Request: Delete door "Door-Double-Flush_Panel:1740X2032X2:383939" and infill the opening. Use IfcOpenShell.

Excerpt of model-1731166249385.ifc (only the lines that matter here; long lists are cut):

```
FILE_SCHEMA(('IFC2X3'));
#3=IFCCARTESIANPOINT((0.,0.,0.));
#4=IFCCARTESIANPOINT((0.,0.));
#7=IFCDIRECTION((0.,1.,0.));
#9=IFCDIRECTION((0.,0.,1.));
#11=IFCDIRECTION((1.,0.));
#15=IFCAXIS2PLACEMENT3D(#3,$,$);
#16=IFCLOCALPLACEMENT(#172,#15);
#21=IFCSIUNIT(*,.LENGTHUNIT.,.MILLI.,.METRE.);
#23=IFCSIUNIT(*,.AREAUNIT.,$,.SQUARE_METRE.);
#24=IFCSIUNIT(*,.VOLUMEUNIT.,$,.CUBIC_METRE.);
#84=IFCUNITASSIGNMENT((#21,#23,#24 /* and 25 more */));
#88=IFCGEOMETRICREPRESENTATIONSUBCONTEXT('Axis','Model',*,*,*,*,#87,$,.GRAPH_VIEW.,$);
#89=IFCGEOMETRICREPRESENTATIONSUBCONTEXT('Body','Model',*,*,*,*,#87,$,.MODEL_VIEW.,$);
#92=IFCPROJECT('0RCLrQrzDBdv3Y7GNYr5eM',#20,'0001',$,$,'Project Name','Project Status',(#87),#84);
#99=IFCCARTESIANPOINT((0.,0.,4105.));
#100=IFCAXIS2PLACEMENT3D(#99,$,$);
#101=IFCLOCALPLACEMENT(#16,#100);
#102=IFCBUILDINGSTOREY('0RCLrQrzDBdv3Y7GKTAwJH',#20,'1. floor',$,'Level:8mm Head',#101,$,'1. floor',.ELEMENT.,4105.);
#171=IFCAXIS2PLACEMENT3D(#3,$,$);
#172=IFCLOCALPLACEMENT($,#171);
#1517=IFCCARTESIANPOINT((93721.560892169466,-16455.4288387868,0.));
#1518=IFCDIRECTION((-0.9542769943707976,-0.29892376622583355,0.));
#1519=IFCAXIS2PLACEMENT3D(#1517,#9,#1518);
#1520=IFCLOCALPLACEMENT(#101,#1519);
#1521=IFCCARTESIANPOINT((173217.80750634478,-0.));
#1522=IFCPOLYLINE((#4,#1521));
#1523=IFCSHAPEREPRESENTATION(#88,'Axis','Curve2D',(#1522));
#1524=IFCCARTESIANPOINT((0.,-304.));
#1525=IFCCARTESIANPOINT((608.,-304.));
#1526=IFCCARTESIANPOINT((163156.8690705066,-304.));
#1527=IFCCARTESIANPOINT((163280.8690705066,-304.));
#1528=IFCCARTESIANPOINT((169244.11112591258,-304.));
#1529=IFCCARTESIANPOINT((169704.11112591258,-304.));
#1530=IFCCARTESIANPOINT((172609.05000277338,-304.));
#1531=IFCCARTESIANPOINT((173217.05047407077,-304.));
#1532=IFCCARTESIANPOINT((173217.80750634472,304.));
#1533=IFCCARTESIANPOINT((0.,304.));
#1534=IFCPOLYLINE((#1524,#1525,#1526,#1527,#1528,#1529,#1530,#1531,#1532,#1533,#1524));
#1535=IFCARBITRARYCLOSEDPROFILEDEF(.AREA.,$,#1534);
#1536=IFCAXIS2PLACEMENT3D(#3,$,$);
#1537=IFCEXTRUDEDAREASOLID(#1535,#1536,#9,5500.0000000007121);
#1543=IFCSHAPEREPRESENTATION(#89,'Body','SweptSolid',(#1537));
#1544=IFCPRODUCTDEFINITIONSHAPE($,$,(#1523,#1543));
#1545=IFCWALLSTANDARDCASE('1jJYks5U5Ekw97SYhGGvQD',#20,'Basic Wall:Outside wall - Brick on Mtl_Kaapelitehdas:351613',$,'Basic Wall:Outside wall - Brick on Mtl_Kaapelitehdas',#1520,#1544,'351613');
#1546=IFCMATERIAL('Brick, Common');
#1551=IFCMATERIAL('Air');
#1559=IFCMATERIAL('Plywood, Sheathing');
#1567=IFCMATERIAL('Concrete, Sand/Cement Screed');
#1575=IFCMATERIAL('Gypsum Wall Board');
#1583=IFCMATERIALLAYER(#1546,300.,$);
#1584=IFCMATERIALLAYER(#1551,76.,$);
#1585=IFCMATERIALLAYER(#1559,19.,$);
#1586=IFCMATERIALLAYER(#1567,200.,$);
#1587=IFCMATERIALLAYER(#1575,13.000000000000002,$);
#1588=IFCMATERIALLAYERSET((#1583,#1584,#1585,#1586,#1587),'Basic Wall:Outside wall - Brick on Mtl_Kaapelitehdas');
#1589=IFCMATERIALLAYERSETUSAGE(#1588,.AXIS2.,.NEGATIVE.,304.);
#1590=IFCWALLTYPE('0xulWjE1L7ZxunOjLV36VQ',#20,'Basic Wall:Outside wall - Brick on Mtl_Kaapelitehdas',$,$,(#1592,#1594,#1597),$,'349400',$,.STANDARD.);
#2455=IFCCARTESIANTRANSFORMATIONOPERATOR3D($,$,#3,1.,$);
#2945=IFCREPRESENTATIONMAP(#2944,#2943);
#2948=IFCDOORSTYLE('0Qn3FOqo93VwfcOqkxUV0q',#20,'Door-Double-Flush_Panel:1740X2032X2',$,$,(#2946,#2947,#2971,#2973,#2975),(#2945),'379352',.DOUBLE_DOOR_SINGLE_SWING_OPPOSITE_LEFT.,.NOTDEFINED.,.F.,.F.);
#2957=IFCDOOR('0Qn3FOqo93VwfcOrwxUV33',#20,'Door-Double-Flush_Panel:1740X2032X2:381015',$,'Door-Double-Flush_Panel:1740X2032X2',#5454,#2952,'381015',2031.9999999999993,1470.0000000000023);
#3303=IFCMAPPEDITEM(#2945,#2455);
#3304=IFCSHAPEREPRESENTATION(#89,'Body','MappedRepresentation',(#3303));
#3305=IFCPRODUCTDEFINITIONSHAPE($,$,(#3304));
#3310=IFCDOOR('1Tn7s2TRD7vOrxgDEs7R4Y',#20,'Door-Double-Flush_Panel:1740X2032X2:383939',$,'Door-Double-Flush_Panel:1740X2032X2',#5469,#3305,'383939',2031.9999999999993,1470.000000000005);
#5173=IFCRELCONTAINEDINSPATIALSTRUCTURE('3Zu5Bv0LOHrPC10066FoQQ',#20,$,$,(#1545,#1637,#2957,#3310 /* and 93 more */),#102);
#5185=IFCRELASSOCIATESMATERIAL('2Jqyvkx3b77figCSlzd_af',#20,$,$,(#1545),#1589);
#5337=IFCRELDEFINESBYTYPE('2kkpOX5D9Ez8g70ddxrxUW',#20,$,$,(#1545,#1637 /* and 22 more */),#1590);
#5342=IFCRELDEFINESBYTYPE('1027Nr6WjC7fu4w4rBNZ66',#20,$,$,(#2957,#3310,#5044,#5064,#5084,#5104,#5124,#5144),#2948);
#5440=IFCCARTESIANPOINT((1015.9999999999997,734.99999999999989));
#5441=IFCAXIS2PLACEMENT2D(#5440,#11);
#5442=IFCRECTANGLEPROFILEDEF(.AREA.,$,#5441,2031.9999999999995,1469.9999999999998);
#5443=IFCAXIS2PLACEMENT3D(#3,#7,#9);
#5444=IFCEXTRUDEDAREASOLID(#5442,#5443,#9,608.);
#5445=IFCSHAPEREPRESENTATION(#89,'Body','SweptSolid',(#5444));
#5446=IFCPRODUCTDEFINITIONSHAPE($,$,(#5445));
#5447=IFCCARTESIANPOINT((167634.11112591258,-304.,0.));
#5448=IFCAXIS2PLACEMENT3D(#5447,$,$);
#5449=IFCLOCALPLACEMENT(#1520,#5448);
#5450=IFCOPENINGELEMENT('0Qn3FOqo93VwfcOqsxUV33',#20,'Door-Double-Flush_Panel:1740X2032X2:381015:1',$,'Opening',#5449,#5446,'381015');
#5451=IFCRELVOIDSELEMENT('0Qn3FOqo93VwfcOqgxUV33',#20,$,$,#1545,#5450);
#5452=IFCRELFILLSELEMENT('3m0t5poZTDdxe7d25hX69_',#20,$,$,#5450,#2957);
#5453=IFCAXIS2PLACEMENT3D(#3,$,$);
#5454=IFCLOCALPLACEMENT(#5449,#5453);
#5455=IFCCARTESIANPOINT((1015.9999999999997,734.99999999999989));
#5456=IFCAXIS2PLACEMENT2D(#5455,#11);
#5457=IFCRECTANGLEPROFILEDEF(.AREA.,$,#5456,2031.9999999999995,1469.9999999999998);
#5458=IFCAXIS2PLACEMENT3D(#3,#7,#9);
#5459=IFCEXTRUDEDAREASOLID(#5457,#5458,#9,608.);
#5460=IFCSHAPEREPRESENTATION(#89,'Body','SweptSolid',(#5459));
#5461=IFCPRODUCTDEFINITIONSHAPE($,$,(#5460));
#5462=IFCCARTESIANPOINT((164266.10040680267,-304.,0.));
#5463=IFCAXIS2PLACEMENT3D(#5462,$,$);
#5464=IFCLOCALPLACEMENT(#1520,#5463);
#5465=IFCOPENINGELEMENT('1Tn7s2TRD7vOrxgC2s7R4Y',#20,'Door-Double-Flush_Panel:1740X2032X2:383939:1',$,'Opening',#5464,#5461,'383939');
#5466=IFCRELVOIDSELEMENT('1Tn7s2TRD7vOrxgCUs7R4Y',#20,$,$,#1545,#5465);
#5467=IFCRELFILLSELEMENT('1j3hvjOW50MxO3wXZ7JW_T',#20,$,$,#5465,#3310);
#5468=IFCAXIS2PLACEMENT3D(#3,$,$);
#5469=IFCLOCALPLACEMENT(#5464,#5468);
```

```python
import ifcopenshell
import ifcopenshell.api.feature
import ifcopenshell.api.root
import ifcopenshell.geom
import ifcopenshell.util.shape

model = ifcopenshell.open("model-1731166249385.ifc")
settings = ifcopenshell.geom.settings()


def volume(element):
    """Net volume in cubic metres, openings subtracted."""
    shape = ifcopenshell.geom.create_shape(settings, element)
    return ifcopenshell.util.shape.get_volume(shape.geometry)


door = model.by_id(3310)
opening = door.FillsVoids[0].RelatingOpeningElement
wall = opening.VoidsElements[0].RelatingBuildingElement
before = volume(wall)

ifcopenshell.api.root.remove_product(model, product=door)
ifcopenshell.api.feature.remove_feature(model, feature=opening)

after = volume(wall)

print(f"wall volume {before:.3f} -> {after:.3f} m3")

model.write("model-1731166249385_v2.ifc")
```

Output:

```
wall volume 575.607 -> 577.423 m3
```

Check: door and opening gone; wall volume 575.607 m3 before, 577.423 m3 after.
